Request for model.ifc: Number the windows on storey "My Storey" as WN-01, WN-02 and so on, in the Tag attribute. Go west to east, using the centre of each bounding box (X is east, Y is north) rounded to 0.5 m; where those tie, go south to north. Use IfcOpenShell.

First a look at what the model holds.

```python
import ifcopenshell
import ifcopenshell.util.element
import ifcopenshell.util.placement

model = ifcopenshell.open("model.ifc")
print(model.schema)
storey = next(s for s in model.by_type("IfcBuildingStorey") if s.Name == "My Storey")
windows = [e for e in ifcopenshell.util.element.get_decomposition(storey) if e.is_a("IfcWindow")]
for e in sorted(windows, key=lambda e: e.id()):
    origin = ifcopenshell.util.placement.get_local_placement(e.ObjectPlacement)[:3, 3]
    print(e.id(), e.Tag, e.Name, origin.round(2) + 0.0, sep=" | ")
```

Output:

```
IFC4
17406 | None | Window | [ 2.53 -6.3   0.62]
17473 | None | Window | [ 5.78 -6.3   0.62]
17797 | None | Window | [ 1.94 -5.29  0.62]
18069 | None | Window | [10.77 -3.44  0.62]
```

```python
import ifcopenshell
import ifcopenshell.geom
import ifcopenshell.util.element
import ifcopenshell.util.shape

model = ifcopenshell.open("model.ifc")
settings = ifcopenshell.geom.settings()
settings.set("use-world-coords", True)


def centre(element):
    shape = ifcopenshell.geom.create_shape(settings, element)
    return ifcopenshell.util.shape.get_bbox_centroid(shape.geometry)


storey = next(s for s in model.by_type("IfcBuildingStorey") if s.Name == "My Storey")
windows = [e for e in ifcopenshell.util.element.get_decomposition(storey) if e.is_a("IfcWindow")]

# Insertion points can sit at a corner or the storey origin, so sort by the geometry (in metres).
centres = {e: centre(e) for e in windows}
windows.sort(key=lambda e: (round(centres[e][0] / 0.5), centres[e][1]))

for i, e in enumerate(windows, start=1):
    number = f"WN-{i:02d}"
    e.Tag = number
    print(e.id(), number)

model.write("model-out.ifc")
```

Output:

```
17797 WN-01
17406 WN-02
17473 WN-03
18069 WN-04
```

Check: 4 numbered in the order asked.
